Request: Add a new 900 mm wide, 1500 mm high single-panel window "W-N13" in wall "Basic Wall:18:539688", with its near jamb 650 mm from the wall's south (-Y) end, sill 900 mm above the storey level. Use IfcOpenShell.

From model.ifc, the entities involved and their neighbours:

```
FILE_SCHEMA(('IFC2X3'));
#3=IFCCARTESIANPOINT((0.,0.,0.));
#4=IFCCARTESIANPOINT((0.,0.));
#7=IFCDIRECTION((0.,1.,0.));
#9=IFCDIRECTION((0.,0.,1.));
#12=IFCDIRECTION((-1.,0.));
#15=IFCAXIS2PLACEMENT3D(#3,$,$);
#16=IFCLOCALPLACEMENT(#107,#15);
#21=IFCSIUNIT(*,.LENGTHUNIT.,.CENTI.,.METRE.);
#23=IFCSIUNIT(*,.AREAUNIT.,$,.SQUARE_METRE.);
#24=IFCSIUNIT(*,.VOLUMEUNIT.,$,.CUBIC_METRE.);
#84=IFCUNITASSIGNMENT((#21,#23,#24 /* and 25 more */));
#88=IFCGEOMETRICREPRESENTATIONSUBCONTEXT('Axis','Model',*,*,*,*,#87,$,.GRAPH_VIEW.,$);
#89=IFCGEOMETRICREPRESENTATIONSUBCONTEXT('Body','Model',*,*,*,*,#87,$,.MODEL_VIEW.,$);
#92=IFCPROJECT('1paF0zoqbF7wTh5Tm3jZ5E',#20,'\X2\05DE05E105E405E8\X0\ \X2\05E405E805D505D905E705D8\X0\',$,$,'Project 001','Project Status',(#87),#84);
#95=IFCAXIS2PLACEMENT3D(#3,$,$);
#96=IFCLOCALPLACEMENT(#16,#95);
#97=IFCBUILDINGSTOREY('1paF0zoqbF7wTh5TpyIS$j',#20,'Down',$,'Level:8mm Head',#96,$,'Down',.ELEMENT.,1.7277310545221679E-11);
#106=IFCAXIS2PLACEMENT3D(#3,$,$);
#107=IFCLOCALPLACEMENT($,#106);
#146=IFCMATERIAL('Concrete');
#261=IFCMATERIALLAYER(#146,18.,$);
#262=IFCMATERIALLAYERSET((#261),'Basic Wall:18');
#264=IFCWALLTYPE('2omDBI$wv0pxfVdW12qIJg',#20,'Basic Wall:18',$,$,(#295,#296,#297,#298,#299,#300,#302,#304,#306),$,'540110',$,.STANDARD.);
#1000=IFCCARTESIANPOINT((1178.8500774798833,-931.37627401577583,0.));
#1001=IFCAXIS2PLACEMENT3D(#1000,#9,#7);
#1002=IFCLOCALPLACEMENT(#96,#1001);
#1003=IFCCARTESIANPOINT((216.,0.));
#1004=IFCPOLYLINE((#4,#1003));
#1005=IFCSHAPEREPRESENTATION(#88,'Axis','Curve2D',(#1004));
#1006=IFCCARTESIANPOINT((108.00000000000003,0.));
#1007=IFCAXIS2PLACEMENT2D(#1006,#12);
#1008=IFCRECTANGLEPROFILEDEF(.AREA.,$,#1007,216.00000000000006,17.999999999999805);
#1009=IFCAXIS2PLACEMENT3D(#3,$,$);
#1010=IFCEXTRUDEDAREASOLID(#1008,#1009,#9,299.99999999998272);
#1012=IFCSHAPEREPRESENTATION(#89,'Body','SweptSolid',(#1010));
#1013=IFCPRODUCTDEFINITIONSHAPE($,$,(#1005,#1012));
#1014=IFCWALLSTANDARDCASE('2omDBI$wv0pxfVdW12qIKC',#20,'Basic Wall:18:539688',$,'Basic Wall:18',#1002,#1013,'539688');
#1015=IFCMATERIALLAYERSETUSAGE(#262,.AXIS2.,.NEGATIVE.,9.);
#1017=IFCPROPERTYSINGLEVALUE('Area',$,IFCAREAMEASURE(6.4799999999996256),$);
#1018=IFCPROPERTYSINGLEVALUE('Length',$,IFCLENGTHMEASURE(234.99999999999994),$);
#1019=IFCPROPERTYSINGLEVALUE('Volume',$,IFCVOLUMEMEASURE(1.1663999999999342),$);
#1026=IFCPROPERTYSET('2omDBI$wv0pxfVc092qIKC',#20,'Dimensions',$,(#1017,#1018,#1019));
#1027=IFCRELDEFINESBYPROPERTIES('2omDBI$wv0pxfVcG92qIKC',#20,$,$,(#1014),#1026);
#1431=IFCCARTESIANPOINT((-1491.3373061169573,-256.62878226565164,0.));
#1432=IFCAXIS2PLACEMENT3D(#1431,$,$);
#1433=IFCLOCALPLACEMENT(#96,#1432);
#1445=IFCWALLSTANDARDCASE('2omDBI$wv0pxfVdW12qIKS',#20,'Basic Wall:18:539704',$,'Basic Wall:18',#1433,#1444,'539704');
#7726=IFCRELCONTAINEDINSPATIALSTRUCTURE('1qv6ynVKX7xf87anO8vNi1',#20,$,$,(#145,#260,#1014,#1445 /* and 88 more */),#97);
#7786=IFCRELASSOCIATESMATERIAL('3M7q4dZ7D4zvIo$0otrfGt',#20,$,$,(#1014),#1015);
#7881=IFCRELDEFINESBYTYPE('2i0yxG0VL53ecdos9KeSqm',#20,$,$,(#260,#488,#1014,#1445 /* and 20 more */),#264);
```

```python
import numpy as np
import ifcopenshell
import ifcopenshell.api.feature
import ifcopenshell.api.geometry
import ifcopenshell.api.pset
import ifcopenshell.api.root
import ifcopenshell.api.spatial
import ifcopenshell.api.type
import ifcopenshell.geom
import ifcopenshell.util.element
import ifcopenshell.util.placement
import ifcopenshell.util.representation
import ifcopenshell.util.shape
import ifcopenshell.util.unit

model = ifcopenshell.open("model.ifc")
unit_scale = ifcopenshell.util.unit.calculate_unit_scale(model)
area_scale = ifcopenshell.util.unit.calculate_unit_scale(model, "AREAUNIT")
volume_scale = ifcopenshell.util.unit.calculate_unit_scale(model, "VOLUMEUNIT")
settings = ifcopenshell.geom.settings()


def volume(element):
    """Net volume in cubic metres, openings subtracted."""
    shape = ifcopenshell.geom.create_shape(settings, element)
    return ifcopenshell.util.shape.get_volume(shape.geometry)


wall = model.by_guid("2omDBI$wv0pxfVdW12qIKC")
storey = ifcopenshell.util.element.get_container(wall, ifc_class="IfcBuildingStorey")
context = ifcopenshell.util.representation.get_context(model, "Model", "Body", "MODEL_VIEW")
before = volume(wall)

width, height, from_end, sill = 0.9, 1.5, 0.65, 0.9  # metres

# The wall runs along its own X axis, and the end named is its -X end.
wall_shape = ifcopenshell.geom.create_shape(settings, wall)
x, y, z = ifcopenshell.util.shape.get_vertices(wall_shape.geometry).T
start = x.min() + from_end
face, thickness = float(y.min()), float(y.max() - y.min())
wall_matrix = ifcopenshell.util.placement.get_local_placement(wall.ObjectPlacement)
level = ifcopenshell.util.placement.get_local_placement(storey.ObjectPlacement)[2, 3]


def in_wall(x, y):
    """Placement at x, y metres in the wall's axes, at sill height."""
    matrix = wall_matrix.copy()
    matrix[:, 3] = wall_matrix @ np.array([x / unit_scale, y / unit_scale, 0.0, 1.0])
    matrix[2, 3] = level + sill / unit_scale
    return matrix


# Opening: a box that overshoots both wall faces by 50 mm.
opening = ifcopenshell.api.root.create_entity(model, ifc_class="IfcOpeningElement")
box = ifcopenshell.api.geometry.add_wall_representation(
    model, context=context, length=width, height=height, thickness=thickness + 0.1
)
ifcopenshell.api.geometry.assign_representation(model, product=opening, representation=box)
ifcopenshell.api.geometry.edit_object_placement(model, product=opening, matrix=in_wall(start, face - 0.05), is_si=False)
ifcopenshell.api.feature.add_feature(model, feature=opening, element=wall)

window = ifcopenshell.api.root.create_entity(model, ifc_class="IfcWindow", name="W-N13")
window.OverallWidth, window.OverallHeight = width / unit_scale, height / unit_scale
body = ifcopenshell.api.geometry.add_window_representation(
    model,
    context=context,
    overall_width=window.OverallWidth,
    overall_height=window.OverallHeight,
    partition_type="SINGLE_PANEL",
)
ifcopenshell.api.geometry.assign_representation(model, product=window, representation=body)
ifcopenshell.api.spatial.assign_container(model, products=[window], relating_structure=storey)
fills = ifcopenshell.api.feature.add_filling(model, opening=opening, element=window)
fills.OwnerHistory = window.OwnerHistory  # required in IFC2X3

# IFC2X3 keeps the operation on the window style.
style = ifcopenshell.api.root.create_entity(model, ifc_class="IfcWindowStyle", name="W-N13")
style.OperationType, style.ConstructionType = "SINGLE_PANEL", "NOTDEFINED"
style.ParameterTakesPrecedence = style.Sizeable = False
ifcopenshell.api.type.assign_type(model, related_objects=[window], relating_type=style)

# Centre the window in the wall's thickness.
ifcopenshell.api.geometry.edit_object_placement(model, product=window, matrix=in_wall(start, face), is_si=False)
window_shape = ifcopenshell.geom.create_shape(settings, window)
depth = ifcopenshell.util.shape.get_vertices(window_shape.geometry)[:, 1]
offset = face + thickness / 2 - (depth.min() + depth.max()) / 2
ifcopenshell.api.geometry.edit_object_placement(model, product=window, matrix=in_wall(start, offset), is_si=False)

after = volume(wall)

# Update the wall's stored quantities.
pset = model.by_id(ifcopenshell.util.element.get_pset(wall, "Dimensions", should_inherit=False)["id"])
ifcopenshell.api.pset.edit_pset(model, pset=pset, properties={
    "Area": model.create_entity("IfcAreaMeasure", after / thickness / area_scale),
    "Volume": model.create_entity("IfcVolumeMeasure", after / volume_scale),
})

print(f"wall volume {before:.3f} -> {after:.3f} m3")

model.write("model_edited.ifc")
```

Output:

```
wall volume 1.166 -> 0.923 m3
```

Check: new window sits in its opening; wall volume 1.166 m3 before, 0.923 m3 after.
